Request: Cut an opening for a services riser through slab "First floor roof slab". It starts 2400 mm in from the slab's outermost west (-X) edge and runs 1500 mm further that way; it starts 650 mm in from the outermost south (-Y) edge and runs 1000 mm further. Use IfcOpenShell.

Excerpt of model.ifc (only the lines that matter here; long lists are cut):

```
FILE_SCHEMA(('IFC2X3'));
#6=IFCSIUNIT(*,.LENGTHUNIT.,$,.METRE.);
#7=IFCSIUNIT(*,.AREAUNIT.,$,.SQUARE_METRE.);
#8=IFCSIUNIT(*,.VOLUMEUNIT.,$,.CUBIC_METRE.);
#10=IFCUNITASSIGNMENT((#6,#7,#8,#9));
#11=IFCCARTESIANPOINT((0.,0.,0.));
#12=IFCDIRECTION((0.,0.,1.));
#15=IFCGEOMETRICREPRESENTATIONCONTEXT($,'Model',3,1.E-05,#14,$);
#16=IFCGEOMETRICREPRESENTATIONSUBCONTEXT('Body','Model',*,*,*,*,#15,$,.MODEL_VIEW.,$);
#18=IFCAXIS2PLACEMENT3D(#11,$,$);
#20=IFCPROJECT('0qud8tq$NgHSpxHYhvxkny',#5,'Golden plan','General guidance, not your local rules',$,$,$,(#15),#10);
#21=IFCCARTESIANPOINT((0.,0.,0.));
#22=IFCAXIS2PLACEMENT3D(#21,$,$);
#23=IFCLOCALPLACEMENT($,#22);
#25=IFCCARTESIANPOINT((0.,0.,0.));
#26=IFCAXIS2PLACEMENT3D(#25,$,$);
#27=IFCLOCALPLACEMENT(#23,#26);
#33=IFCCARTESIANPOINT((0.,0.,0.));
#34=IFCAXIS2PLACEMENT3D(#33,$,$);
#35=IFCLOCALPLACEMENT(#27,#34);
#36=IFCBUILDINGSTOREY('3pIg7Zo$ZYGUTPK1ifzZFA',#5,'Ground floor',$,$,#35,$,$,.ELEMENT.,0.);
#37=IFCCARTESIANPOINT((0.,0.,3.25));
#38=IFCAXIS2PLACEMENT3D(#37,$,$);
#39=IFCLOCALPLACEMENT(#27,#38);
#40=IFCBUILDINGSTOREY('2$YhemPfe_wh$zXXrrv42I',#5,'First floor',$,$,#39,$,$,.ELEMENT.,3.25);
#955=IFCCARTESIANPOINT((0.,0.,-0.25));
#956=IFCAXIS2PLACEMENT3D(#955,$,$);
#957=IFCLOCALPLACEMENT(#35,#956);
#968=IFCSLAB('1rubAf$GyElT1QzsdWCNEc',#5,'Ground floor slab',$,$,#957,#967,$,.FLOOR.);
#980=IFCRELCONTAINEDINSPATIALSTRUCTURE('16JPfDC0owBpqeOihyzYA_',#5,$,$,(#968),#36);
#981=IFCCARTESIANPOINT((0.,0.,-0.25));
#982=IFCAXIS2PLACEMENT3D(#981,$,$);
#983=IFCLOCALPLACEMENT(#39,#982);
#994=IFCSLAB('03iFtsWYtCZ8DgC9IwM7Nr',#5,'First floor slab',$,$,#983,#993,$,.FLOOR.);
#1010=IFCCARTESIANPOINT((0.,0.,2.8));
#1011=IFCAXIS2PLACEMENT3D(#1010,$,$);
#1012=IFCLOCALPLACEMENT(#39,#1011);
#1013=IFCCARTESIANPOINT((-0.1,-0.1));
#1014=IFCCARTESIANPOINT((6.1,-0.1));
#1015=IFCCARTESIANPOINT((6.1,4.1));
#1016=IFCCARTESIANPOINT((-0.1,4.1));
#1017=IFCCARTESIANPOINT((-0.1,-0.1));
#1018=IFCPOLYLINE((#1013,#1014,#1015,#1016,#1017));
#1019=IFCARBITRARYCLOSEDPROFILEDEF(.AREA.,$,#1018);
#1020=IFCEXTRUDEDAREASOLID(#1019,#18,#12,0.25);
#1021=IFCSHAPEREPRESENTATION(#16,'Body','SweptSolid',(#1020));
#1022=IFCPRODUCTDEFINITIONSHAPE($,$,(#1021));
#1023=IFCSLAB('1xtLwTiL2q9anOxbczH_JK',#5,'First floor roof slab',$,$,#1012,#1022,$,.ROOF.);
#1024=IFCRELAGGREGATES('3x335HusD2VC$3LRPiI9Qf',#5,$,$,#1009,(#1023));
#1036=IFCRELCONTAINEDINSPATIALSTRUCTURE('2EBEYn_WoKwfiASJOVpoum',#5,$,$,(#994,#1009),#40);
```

```python
import numpy as np
import ifcopenshell
import ifcopenshell.api.feature
import ifcopenshell.api.geometry
import ifcopenshell.api.root
import ifcopenshell.geom
import ifcopenshell.util.placement
import ifcopenshell.util.representation
import ifcopenshell.util.shape
import ifcopenshell.util.unit

model = ifcopenshell.open("model.ifc")
unit_scale = ifcopenshell.util.unit.calculate_unit_scale(model)
settings = ifcopenshell.geom.settings()


def volume(element):
    """Net volume in cubic metres, openings subtracted."""
    shape = ifcopenshell.geom.create_shape(settings, element)
    return ifcopenshell.util.shape.get_volume(shape.geometry)


slab = model.by_id(1023)
before = volume(slab)

# Extent in the slab's own axes, in metres. The edges named are its -X and -Y sides.
slab_shape = ifcopenshell.geom.create_shape(settings, slab)
vertices = ifcopenshell.util.shape.get_vertices(slab_shape.geometry)
x_min, y_min, bottom = vertices.min(axis=0)
top = vertices[:, 2].max()

opening = ifcopenshell.api.root.create_entity(model, ifc_class="IfcOpeningElement", name="Services riser opening")
context = ifcopenshell.util.representation.get_context(model, "Model", "Body", "MODEL_VIEW")
width, depth = 1.5, 1
outline = [(0.0, 0.0), (width, 0.0), (width, depth), (0.0, depth), (0.0, 0.0)]
# Overshoot both faces by 50 mm so the cut is clean.
shape = ifcopenshell.api.geometry.add_slab_representation(
    model, context=context, depth=top - bottom + 0.1, polyline=outline
)
ifcopenshell.api.geometry.assign_representation(model, product=opening, representation=shape)

matrix = ifcopenshell.util.placement.get_local_placement(slab.ObjectPlacement)
matrix[:, 3] = matrix @ np.append(np.array([x_min + 2.4, y_min + 0.65, bottom - 0.05]) / unit_scale, 1.0)
ifcopenshell.api.geometry.edit_object_placement(model, product=opening, matrix=matrix, is_si=False)
ifcopenshell.api.feature.add_feature(model, feature=opening, element=slab)

after = volume(slab)

print(f"slab volume {before:.3f} -> {after:.3f} m3")

model.write("model_v2.ifc")
```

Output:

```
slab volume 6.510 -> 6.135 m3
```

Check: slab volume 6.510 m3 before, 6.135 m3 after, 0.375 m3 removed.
